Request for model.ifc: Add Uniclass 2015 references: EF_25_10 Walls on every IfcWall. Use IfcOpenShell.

First a look at what the model holds.

```python
import ifcopenshell

model = ifcopenshell.open("model.ifc")
print(model.schema)
print("classifications:", [c.Name for c in model.by_type("IfcClassification")])
for ifc_class in ("IfcDoor", "IfcRoof", "IfcStair", "IfcWall", "IfcWindow"):
    print(ifc_class, len(model.by_type(ifc_class)))
```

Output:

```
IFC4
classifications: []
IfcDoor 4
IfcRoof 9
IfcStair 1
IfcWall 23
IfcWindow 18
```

```python
import ifcopenshell
import ifcopenshell.api.classification

model = ifcopenshell.open("model.ifc")

system = ifcopenshell.api.classification.add_classification(model, classification="Uniclass 2015")

codes = {
    "IfcWall": ("EF_25_10", "Walls"),
}
for ifc_class, (code, name) in codes.items():
    products = model.by_type(ifc_class)
    ifcopenshell.api.classification.add_reference(
        model, products=products, classification=system, identification=code, name=name
    )
    print(code, len(products))

model.write("model_rev.ifc")
```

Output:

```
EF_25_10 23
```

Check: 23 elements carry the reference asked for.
